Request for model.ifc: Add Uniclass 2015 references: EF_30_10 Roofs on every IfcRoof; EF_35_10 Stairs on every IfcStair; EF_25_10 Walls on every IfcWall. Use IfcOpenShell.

First a look at what the model holds.

```python
import ifcopenshell

model = ifcopenshell.open("model.ifc")
print(model.schema)
print("classifications:", [c.Name for c in model.by_type("IfcClassification")])
for ifc_class in ("IfcDoor", "IfcRoof", "IfcStair", "IfcWall", "IfcWindow"):
    print(ifc_class, len(model.by_type(ifc_class)))
```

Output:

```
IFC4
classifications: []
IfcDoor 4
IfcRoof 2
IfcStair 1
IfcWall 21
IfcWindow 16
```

```python
import ifcopenshell
import ifcopenshell.api.classification

model = ifcopenshell.open("model.ifc")

system = ifcopenshell.api.classification.add_classification(model, classification="Uniclass 2015")

codes = {
    "IfcRoof": ("EF_30_10", "Roofs"),
    "IfcStair": ("EF_35_10", "Stairs"),
    "IfcWall": ("EF_25_10", "Walls"),
}
for ifc_class, (code, name) in codes.items():
    products = model.by_type(ifc_class)
    ifcopenshell.api.classification.add_reference(
        model, products=products, classification=system, identification=code, name=name
    )
    print(code, len(products))

model.write("model_v2.ifc")
```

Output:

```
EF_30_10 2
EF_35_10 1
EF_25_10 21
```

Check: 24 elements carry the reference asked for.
